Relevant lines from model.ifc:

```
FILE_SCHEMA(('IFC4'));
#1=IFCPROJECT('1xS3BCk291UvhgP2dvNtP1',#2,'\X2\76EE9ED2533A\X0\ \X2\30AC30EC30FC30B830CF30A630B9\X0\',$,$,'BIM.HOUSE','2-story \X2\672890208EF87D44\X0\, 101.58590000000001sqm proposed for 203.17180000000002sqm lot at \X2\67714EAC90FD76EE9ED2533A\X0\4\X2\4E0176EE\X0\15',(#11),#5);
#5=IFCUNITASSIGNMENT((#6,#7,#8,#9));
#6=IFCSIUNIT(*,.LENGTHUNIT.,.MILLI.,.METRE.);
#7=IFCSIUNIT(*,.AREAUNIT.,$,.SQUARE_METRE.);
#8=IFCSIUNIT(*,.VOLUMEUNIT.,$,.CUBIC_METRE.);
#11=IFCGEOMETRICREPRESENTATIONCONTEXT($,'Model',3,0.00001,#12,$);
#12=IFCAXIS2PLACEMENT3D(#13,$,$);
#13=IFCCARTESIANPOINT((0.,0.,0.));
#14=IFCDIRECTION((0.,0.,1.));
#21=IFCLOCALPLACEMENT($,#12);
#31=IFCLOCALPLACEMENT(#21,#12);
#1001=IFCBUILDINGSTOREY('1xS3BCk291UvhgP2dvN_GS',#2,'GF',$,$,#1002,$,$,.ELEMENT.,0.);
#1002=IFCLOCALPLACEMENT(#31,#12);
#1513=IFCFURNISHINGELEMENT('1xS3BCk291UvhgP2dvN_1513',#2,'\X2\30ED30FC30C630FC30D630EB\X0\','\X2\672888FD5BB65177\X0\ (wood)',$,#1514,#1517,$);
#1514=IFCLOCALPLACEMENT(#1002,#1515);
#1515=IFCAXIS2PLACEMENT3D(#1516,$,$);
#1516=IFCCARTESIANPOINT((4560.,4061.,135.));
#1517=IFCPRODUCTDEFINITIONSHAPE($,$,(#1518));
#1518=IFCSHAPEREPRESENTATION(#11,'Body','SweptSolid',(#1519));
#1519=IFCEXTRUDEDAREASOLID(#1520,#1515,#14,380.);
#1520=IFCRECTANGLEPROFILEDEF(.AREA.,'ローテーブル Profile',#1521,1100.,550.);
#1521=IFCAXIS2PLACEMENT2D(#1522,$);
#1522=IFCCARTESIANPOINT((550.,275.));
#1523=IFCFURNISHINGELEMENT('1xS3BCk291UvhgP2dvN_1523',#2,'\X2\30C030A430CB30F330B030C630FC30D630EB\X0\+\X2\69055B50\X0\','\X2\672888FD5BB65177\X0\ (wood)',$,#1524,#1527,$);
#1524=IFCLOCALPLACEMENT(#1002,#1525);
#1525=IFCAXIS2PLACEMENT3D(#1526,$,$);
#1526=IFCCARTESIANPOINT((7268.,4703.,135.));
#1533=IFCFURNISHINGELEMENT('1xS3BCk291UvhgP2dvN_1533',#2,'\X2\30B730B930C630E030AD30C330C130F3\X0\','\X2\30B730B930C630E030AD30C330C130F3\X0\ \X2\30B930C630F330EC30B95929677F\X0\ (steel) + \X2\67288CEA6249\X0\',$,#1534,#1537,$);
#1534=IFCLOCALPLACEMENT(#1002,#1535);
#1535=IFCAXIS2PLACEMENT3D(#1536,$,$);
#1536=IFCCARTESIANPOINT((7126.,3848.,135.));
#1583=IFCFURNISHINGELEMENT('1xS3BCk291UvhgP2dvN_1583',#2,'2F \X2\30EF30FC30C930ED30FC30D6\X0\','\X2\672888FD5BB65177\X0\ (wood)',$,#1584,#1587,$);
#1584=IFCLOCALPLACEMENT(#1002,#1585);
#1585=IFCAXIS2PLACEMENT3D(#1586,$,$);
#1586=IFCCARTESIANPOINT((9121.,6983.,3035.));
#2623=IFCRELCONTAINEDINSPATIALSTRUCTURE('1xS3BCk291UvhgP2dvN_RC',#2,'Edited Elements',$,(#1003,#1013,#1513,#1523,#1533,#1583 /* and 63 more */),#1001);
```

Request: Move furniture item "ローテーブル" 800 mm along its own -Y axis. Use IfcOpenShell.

```python
import ifcopenshell
import ifcopenshell.api.geometry
import ifcopenshell.util.placement
import ifcopenshell.util.unit

model = ifcopenshell.open("model.ifc")
unit_scale = ifcopenshell.util.unit.calculate_unit_scale(model)

item = model.by_guid("1xS3BCk291UvhgP2dvN_1513")
matrix = ifcopenshell.util.placement.get_local_placement(item.ObjectPlacement)
matrix[:3, 3] -= matrix[:3, 1] * 0.8 / unit_scale
ifcopenshell.api.geometry.edit_object_placement(model, product=item, matrix=matrix, is_si=False)

print(ifcopenshell.util.placement.get_local_placement(item.ObjectPlacement).round(3) + 0.0)

model.write("model_v2.ifc")
```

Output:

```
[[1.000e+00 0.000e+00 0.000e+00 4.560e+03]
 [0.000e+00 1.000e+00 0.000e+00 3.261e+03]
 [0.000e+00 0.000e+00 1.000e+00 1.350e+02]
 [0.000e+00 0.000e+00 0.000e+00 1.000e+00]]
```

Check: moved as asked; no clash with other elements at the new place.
